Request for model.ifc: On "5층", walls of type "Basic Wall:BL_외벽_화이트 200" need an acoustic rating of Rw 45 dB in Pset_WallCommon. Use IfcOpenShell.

First a look at what the model holds.

```python
import ifcopenshell
import ifcopenshell.util.element

model = ifcopenshell.open("model.ifc")
print(model.schema)
storey = next(s for s in model.by_type("IfcBuildingStorey") if s.Name == "5층")
walls = [e for e in ifcopenshell.util.element.get_decomposition(storey) if e.is_a("IfcWall")]
seen = {}
for e in walls:
    element_type = ifcopenshell.util.element.get_type(e)
    key = (element_type.Name if element_type != e and element_type else None, ifcopenshell.util.element.get_pset(e, "Pset_WallCommon", "AcousticRating"))
    seen[key] = seen.get(key, 0) + 1
for (name, value), count in sorted(seen.items(), key=str):
    print(count, "x", name, "|", value)
```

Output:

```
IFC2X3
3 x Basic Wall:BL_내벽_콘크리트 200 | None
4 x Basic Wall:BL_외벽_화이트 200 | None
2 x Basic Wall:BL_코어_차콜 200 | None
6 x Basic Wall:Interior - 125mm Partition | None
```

```python
import ifcopenshell
import ifcopenshell.api.pset
import ifcopenshell.util.element

model = ifcopenshell.open("model.ifc")

storey = next(s for s in model.by_type("IfcBuildingStorey") if s.Name == "5층")
walls = [e for e in ifcopenshell.util.element.get_decomposition(storey) if e.is_a("IfcWall")]

count = 0
for e in walls:
    element_type = ifcopenshell.util.element.get_type(e)
    if element_type in (None, e) or element_type.Name != "Basic Wall:BL_외벽_화이트 200":
        continue
    # add_pset returns the element's existing set when there is one.
    pset = ifcopenshell.api.pset.add_pset(model, product=e, name="Pset_WallCommon")
    ifcopenshell.api.pset.edit_pset(model, pset=pset, properties={"AcousticRating": "Rw 45 dB"})
    count += 1

print(count, "walls updated")

model.write("model_edited.ifc")
```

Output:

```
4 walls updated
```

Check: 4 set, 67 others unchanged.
